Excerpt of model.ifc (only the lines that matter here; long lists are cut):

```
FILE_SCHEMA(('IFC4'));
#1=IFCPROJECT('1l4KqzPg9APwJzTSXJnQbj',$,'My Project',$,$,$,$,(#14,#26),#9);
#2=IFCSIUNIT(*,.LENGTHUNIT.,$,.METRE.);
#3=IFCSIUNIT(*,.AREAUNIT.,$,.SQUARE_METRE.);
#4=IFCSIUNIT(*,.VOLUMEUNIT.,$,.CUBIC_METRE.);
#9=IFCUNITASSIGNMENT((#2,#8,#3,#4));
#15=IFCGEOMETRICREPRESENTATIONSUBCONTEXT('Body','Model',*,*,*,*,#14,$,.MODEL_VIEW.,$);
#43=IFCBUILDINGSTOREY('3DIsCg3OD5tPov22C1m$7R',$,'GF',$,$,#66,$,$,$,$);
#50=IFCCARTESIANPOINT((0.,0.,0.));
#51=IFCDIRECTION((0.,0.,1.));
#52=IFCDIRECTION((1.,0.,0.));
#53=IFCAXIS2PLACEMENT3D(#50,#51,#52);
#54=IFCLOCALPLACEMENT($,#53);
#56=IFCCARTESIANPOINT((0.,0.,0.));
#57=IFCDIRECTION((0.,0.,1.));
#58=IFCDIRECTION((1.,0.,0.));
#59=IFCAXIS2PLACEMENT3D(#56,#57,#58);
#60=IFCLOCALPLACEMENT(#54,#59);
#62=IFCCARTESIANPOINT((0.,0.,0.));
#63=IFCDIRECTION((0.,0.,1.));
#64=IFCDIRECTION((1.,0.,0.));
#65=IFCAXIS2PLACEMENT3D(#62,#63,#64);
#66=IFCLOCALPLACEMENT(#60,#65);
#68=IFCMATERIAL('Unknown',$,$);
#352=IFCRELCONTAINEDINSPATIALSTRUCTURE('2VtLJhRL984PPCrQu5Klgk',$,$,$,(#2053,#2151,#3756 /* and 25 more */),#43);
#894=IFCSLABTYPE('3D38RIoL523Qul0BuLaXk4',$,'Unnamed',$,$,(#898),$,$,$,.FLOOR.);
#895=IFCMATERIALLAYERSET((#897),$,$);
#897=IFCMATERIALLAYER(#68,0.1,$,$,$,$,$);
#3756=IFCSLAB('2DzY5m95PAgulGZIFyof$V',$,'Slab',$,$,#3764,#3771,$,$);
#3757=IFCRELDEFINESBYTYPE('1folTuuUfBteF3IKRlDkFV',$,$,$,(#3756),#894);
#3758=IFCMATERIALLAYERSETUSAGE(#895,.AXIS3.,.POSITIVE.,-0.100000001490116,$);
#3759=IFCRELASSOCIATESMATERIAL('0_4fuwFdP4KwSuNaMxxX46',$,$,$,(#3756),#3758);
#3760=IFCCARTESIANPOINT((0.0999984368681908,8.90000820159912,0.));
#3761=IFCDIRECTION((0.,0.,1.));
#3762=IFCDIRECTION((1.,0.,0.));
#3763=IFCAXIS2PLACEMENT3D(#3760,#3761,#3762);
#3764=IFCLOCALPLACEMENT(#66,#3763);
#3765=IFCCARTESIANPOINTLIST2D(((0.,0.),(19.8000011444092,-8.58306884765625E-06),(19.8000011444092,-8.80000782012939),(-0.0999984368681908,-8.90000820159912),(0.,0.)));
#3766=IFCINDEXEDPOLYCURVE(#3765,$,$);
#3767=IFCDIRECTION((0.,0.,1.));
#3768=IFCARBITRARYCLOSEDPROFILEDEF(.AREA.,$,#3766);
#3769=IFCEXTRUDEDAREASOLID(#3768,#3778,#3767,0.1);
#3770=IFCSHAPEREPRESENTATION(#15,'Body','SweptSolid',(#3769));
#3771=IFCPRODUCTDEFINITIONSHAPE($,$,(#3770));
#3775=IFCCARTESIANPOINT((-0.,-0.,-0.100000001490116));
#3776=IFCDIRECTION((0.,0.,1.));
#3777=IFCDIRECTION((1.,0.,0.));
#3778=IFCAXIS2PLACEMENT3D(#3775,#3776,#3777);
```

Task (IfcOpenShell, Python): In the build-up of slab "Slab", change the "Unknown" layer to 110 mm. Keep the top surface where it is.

```python
import ifcopenshell
import ifcopenshell.util.element
import ifcopenshell.util.representation
import ifcopenshell.util.unit

model = ifcopenshell.open("model.ifc")
unit_scale = ifcopenshell.util.unit.calculate_unit_scale(model)

layer_set = model.by_id(895)
layer = next(l for l in layer_set.MaterialLayers if l.Material and l.Material.Name == "Unknown")
change = 0.11 / unit_scale - layer.LayerThickness
layer.LayerThickness += change

# Geometry does not follow the layer set by itself.
slabs = [e for e in ifcopenshell.util.element.get_elements_by_material(model, layer_set) if e.is_a("IfcSlab")]
for slab in sorted(slabs, key=lambda e: e.id()):
    body = ifcopenshell.util.representation.get_representation(slab, "Model", "Body")
    solid = body.Items[0]
    old_depth = solid.Depth
    solid.Depth += change
    # Extruded upwards: lower the start of the extrusion so the top stays.
    x, y, z = solid.Position.Location.Coordinates
    solid.Position.Location = model.createIfcCartesianPoint((x, y, z - change))
    print(slab.id(), f"{old_depth:g} -> {solid.Depth:g}")

# The layers are counted up from the underside, which has moved.
for usage in {ifcopenshell.util.element.get_material(slab) for slab in slabs}:
    usage.OffsetFromReferenceLine -= change

model.write("model_edited.ifc")
```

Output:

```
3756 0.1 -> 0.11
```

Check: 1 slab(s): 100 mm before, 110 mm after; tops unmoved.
